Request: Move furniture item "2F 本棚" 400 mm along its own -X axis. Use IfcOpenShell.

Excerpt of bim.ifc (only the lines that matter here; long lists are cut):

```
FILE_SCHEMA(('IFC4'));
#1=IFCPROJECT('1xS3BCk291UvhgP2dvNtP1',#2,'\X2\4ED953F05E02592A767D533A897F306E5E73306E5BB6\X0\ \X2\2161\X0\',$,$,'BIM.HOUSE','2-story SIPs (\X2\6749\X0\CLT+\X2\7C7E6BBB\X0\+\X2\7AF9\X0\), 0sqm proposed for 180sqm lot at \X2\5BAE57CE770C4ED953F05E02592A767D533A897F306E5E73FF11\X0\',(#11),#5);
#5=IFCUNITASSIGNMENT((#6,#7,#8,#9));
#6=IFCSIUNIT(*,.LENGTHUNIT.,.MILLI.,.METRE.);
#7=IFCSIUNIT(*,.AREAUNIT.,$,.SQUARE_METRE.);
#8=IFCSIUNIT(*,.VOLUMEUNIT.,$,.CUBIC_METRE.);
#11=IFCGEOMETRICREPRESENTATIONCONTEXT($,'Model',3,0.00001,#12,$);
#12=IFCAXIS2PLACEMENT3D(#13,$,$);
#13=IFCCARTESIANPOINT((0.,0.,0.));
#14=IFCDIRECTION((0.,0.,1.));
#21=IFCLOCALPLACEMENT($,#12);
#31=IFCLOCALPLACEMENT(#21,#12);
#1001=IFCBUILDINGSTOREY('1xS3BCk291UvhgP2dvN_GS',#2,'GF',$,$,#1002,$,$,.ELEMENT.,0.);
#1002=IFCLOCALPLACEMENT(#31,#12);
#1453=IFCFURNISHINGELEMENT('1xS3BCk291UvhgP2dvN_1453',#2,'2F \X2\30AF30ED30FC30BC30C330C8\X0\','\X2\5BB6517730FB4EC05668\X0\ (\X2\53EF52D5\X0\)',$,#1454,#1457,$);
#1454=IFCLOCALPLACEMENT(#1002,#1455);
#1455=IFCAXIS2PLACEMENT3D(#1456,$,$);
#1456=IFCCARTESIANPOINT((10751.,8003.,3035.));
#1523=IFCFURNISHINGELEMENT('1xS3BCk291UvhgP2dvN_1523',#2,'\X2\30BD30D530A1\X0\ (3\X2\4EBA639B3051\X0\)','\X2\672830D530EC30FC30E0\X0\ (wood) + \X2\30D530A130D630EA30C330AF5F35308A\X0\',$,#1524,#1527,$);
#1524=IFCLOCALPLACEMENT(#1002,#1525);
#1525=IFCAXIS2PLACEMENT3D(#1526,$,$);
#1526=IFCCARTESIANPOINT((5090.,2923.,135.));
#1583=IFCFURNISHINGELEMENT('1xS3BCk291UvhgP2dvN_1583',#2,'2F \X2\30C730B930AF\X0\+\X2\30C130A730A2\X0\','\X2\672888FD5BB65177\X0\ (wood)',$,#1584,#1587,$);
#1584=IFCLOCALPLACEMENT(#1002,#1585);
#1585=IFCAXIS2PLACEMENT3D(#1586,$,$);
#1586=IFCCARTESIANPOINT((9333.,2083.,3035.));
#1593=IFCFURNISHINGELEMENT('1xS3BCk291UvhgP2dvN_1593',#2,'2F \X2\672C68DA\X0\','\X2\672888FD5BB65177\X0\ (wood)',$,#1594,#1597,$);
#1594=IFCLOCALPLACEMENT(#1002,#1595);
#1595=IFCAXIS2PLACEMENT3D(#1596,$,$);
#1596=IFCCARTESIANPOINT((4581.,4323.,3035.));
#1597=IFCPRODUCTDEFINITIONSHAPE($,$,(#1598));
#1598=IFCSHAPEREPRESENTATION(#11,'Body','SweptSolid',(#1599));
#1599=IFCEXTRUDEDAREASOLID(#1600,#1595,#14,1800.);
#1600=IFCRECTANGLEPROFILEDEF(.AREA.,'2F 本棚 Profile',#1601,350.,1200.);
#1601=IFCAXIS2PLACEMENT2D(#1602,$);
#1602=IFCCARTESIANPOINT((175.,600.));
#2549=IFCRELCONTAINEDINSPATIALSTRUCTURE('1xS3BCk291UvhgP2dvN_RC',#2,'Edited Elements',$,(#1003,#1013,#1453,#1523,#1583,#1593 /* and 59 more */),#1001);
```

```python
import ifcopenshell
import ifcopenshell.api.geometry
import ifcopenshell.util.placement

model = ifcopenshell.open("bim.ifc")

item = model.by_guid("1xS3BCk291UvhgP2dvN_1593")
matrix = ifcopenshell.util.placement.get_local_placement(item.ObjectPlacement)
matrix[:3, 3] -= matrix[:3, 0] * 400.0
ifcopenshell.api.geometry.edit_object_placement(model, product=item, matrix=matrix, is_si=False)

print(ifcopenshell.util.placement.get_local_placement(item.ObjectPlacement).round(3) + 0.0)

model.write("bim_v2.ifc")
```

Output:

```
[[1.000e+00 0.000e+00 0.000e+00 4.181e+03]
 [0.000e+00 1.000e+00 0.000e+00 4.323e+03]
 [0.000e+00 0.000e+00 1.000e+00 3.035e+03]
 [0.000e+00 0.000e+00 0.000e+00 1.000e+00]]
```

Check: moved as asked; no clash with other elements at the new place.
